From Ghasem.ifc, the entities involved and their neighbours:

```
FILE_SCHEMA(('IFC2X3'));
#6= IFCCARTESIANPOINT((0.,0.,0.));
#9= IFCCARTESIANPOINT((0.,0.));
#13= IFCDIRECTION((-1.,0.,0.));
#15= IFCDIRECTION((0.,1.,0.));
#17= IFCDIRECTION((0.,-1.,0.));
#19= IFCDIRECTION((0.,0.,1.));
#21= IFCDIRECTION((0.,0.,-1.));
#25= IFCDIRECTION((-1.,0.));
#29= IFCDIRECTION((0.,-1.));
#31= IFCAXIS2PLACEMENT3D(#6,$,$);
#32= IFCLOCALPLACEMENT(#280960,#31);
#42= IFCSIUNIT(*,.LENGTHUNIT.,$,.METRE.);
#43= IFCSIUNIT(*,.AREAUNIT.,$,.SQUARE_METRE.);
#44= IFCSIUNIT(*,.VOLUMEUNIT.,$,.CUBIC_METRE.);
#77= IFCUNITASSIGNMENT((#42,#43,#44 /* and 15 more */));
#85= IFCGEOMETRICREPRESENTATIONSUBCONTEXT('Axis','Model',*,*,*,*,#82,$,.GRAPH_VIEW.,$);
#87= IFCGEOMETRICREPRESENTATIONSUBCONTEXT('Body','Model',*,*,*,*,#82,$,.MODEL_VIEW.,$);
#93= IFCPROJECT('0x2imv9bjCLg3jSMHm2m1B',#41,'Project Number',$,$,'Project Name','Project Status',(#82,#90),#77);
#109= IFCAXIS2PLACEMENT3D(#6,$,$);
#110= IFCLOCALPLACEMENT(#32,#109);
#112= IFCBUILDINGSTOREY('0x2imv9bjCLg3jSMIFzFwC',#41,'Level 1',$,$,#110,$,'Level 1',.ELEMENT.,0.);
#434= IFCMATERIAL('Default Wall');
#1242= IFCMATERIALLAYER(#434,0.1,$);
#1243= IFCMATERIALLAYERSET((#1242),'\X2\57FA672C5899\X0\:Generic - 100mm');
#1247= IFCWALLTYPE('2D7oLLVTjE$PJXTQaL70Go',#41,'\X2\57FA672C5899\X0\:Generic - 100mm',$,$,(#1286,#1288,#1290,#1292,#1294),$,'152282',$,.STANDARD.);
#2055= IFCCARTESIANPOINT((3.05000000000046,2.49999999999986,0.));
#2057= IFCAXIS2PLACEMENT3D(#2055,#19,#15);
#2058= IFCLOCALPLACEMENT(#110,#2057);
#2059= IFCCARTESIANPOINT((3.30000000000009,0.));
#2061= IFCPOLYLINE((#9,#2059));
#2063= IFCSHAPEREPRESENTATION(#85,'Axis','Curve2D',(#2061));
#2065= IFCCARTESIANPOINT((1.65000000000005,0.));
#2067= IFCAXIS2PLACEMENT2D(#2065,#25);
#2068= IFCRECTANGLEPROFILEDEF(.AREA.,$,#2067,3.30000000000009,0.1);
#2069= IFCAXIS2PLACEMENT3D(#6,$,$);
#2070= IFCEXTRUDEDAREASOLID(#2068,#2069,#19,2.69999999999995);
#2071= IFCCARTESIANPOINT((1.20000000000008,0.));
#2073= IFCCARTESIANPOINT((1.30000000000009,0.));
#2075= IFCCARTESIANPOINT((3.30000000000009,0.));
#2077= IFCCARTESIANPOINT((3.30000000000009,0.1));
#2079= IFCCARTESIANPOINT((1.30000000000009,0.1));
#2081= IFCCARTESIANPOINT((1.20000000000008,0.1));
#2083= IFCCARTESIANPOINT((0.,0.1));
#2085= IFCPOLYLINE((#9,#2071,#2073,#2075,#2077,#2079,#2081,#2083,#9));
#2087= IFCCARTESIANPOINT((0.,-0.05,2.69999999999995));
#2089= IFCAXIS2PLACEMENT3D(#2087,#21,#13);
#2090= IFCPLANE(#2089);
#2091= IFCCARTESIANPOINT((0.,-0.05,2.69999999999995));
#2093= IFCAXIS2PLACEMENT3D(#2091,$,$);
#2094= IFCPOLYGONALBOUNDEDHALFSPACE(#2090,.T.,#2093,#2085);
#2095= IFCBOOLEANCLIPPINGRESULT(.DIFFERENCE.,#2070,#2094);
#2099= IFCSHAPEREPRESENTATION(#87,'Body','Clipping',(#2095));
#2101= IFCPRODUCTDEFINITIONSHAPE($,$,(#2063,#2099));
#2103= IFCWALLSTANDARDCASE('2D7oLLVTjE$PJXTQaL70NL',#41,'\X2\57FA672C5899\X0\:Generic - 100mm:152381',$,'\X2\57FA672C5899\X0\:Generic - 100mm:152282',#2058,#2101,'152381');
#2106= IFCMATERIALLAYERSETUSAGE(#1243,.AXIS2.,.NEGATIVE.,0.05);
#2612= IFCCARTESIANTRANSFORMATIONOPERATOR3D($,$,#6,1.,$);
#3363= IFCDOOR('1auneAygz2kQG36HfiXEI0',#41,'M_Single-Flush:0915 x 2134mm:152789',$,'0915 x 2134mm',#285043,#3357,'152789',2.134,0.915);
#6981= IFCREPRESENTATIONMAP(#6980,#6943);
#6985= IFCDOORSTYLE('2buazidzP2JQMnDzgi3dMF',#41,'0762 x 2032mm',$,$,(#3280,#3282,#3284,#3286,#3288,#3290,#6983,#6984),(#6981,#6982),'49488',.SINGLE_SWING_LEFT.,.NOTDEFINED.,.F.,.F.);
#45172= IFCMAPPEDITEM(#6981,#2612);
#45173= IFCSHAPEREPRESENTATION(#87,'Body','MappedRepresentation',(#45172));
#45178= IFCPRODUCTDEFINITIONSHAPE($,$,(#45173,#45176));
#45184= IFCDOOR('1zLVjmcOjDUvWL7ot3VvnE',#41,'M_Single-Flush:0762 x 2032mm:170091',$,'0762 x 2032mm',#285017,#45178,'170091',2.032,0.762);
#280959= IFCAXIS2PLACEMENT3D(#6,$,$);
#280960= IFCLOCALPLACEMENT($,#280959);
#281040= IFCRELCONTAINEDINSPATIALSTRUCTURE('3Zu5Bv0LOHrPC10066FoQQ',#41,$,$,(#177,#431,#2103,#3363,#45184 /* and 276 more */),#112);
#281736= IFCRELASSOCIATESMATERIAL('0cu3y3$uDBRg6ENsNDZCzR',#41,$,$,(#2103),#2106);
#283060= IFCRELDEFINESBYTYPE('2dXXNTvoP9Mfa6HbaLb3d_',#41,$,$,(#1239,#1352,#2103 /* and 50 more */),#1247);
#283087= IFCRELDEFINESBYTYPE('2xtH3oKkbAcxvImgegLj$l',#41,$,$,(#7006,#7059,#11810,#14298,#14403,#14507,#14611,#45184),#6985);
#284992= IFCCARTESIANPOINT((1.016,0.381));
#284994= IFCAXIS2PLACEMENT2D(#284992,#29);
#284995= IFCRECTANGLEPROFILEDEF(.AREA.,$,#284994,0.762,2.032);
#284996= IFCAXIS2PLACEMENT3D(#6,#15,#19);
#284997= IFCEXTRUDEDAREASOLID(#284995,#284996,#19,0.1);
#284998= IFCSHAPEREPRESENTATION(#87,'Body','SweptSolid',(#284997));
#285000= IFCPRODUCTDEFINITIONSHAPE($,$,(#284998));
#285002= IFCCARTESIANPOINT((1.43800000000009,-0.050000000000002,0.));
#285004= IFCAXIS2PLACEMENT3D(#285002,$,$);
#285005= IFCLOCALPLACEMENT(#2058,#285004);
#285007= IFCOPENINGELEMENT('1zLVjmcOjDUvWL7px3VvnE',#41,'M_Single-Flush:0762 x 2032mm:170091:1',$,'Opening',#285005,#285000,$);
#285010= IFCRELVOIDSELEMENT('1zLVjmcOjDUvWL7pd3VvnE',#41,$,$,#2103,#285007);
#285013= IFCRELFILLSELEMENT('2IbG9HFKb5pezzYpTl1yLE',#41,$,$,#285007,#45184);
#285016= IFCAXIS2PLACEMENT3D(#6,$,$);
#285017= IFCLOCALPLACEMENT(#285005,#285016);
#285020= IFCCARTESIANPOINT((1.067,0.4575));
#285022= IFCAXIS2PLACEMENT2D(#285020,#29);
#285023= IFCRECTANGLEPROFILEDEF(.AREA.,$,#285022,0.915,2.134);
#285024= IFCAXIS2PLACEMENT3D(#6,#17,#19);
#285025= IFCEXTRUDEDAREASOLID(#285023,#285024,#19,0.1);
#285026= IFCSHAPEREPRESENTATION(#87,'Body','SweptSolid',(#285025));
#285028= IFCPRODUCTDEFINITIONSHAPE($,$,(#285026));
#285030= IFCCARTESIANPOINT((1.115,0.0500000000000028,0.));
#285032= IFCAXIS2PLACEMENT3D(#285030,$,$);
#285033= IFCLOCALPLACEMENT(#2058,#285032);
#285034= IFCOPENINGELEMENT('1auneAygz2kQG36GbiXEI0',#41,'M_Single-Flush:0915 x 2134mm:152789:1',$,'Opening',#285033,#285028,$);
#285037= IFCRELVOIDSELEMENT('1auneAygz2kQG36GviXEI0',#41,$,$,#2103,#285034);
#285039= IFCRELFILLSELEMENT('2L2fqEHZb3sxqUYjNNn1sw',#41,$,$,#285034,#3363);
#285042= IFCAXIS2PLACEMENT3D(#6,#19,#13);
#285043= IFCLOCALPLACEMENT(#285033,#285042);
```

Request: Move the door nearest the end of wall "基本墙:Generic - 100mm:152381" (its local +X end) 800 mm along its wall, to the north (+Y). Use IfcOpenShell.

```python
import ifcopenshell
import ifcopenshell.api.geometry
import ifcopenshell.util.placement
import ifcopenshell.util.unit

model = ifcopenshell.open("Ghasem.ifc")
unit_scale = ifcopenshell.util.unit.calculate_unit_scale(model)

door = model.by_id(45184)
opening = door.FillsVoids[0].RelatingOpeningElement
wall = opening.VoidsElements[0].RelatingBuildingElement

wall_matrix = ifcopenshell.util.placement.get_local_placement(wall.ObjectPlacement)
shift = wall_matrix[:3, 0] * 0.8 / unit_scale
before = ifcopenshell.util.placement.get_local_placement(door.ObjectPlacement)[:3, 3].copy()

# The door is placed relative to its opening, so it follows when the opening moves.
matrix = ifcopenshell.util.placement.get_local_placement(opening.ObjectPlacement)
matrix[:3, 3] += shift
ifcopenshell.api.geometry.edit_object_placement(
    model, product=opening, matrix=matrix, is_si=False, should_transform_children=True
)

after = ifcopenshell.util.placement.get_local_placement(door.ObjectPlacement)[:3, 3]
print("door moved by", (after - before).round(3) + 0.0)

model.write("Ghasem_updated.ifc")
```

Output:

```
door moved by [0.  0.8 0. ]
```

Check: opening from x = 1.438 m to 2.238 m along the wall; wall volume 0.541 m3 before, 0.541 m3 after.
